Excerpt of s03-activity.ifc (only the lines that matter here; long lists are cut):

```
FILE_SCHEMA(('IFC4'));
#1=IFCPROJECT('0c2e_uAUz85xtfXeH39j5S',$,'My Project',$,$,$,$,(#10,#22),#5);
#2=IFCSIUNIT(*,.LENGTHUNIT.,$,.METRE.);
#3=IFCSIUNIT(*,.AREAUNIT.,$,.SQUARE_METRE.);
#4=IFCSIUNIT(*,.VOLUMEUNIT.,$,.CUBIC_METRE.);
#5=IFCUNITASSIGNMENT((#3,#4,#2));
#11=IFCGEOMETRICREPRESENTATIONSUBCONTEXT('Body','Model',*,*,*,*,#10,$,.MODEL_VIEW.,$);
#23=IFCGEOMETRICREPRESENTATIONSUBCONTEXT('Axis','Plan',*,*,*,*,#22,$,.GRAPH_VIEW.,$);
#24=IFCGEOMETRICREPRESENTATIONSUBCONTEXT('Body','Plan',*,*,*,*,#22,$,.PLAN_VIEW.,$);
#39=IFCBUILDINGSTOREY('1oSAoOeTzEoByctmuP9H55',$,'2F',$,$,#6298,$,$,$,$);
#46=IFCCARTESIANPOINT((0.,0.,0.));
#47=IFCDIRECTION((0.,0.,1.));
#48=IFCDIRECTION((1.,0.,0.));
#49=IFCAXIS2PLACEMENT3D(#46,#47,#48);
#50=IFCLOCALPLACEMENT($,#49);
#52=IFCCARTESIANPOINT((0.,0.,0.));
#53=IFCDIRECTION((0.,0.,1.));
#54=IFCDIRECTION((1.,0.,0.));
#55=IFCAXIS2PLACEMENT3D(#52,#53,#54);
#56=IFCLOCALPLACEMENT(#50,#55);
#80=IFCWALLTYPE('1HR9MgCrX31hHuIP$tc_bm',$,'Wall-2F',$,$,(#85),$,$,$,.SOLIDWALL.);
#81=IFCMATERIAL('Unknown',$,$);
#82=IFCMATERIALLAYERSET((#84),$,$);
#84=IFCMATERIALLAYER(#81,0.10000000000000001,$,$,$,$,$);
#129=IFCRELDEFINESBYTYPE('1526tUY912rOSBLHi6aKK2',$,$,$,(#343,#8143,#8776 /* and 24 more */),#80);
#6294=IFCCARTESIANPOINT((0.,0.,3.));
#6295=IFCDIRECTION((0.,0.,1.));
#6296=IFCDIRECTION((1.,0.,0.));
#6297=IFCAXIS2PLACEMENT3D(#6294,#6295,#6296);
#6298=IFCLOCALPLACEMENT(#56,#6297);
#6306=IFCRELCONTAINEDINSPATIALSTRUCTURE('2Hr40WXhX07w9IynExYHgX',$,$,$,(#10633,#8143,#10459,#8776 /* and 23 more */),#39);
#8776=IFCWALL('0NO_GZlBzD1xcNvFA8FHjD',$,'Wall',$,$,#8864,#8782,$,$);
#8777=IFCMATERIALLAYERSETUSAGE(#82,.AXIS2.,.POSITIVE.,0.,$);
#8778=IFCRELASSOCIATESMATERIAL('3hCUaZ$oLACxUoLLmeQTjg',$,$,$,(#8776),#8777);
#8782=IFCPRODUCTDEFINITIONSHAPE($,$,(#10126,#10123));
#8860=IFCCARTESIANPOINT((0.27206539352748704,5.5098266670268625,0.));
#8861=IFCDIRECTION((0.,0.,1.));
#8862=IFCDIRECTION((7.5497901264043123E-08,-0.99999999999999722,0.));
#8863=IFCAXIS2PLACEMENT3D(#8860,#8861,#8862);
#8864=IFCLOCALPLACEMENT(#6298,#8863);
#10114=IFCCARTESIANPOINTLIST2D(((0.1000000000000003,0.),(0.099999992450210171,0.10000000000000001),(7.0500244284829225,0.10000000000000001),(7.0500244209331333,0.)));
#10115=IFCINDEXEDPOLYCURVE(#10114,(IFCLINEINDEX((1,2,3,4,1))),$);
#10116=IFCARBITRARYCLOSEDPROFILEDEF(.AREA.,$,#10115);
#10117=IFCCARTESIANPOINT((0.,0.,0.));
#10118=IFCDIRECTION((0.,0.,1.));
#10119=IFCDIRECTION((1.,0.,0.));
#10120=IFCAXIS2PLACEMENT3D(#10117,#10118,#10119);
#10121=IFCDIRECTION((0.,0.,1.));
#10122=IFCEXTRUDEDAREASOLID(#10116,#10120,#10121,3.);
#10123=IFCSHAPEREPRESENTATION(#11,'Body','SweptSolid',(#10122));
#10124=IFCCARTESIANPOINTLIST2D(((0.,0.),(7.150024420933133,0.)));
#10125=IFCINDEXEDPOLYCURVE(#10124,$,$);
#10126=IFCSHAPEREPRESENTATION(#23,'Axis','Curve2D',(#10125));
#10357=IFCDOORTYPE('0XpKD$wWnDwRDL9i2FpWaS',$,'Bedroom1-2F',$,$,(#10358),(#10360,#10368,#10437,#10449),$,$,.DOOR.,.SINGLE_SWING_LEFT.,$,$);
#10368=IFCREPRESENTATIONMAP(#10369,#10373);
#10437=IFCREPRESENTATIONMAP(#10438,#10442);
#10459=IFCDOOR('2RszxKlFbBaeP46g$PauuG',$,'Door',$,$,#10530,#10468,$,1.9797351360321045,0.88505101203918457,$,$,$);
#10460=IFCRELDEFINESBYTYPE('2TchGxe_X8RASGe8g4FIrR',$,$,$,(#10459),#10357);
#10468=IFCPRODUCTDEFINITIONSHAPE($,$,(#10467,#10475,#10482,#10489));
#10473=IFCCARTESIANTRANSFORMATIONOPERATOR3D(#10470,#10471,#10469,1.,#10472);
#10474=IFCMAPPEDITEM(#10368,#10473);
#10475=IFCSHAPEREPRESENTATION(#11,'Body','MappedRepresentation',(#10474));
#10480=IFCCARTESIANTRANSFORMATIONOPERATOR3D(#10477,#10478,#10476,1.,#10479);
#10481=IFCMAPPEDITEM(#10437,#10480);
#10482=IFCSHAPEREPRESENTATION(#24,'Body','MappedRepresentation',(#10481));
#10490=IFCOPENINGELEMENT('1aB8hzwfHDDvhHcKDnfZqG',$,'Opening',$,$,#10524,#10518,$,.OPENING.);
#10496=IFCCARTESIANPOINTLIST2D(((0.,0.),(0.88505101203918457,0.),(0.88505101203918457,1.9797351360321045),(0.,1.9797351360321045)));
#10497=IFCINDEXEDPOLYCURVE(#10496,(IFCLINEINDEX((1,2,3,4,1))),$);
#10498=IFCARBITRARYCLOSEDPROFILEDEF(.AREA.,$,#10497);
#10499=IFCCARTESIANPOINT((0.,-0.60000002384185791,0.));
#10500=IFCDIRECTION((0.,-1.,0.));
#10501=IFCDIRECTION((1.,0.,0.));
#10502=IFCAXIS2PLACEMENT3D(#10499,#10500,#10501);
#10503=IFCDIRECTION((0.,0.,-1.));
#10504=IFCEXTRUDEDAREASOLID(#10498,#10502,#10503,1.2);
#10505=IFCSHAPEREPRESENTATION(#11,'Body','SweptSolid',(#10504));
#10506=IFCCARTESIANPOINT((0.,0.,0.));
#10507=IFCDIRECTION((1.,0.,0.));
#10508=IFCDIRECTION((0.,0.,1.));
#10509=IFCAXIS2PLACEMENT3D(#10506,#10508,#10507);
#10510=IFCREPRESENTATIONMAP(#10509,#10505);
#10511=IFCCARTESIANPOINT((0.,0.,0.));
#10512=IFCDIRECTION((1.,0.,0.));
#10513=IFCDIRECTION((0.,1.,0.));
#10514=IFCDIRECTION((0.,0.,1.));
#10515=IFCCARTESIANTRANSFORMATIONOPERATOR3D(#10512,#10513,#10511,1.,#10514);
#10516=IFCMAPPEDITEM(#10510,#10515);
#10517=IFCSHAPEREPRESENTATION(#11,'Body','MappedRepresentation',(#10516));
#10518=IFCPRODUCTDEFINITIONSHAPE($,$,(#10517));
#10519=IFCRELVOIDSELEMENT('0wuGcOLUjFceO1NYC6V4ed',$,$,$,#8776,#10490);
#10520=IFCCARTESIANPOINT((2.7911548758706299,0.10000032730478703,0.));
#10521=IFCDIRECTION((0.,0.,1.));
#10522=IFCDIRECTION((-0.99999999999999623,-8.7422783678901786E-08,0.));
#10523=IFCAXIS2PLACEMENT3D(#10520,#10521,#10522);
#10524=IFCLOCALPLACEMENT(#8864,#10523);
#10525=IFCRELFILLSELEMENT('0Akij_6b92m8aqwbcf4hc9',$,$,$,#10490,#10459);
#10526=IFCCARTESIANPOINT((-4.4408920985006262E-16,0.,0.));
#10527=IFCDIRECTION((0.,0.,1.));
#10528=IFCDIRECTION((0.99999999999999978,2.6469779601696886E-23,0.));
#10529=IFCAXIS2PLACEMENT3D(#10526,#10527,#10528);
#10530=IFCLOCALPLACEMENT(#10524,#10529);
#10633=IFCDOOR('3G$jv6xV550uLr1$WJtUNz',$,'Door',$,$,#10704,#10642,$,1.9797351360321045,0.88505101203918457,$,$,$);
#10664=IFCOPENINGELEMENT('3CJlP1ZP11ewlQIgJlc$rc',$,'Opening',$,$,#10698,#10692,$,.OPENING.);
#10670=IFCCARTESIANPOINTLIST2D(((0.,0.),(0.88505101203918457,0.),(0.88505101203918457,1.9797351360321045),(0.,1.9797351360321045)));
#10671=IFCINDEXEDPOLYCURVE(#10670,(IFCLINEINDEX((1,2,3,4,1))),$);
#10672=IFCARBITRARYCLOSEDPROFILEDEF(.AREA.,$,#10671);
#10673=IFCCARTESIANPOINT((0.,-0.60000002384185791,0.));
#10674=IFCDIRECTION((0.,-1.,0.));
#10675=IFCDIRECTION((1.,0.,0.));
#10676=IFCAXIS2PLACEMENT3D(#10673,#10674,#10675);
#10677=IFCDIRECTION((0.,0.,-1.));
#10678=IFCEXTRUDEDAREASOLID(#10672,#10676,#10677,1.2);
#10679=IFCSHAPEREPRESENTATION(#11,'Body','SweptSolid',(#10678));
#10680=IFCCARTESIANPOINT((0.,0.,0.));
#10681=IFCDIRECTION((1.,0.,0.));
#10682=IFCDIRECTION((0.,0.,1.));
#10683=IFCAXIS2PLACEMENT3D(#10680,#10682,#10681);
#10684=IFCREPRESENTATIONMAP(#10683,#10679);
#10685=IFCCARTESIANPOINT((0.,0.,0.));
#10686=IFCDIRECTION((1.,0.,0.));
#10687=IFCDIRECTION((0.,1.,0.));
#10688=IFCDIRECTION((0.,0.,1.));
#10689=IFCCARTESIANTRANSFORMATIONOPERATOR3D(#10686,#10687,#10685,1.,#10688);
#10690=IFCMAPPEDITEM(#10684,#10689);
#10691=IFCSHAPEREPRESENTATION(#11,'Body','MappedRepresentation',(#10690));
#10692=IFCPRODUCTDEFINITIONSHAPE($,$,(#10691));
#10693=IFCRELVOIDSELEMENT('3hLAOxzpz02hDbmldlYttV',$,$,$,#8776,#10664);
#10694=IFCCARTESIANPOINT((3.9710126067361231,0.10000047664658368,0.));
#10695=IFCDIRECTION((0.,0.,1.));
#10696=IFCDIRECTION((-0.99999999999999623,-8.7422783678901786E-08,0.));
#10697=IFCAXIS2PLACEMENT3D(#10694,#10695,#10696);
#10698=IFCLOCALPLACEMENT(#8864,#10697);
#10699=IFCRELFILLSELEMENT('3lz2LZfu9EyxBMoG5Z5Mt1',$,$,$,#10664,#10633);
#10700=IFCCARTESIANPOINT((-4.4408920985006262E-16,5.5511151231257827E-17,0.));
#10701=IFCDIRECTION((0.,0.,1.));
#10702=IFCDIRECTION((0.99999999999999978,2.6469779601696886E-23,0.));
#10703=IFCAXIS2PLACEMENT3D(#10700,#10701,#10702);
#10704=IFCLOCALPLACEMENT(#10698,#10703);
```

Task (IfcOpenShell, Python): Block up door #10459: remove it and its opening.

```python
import ifcopenshell
import ifcopenshell.api.feature
import ifcopenshell.api.root
import ifcopenshell.geom
import ifcopenshell.util.shape

model = ifcopenshell.open("s03-activity.ifc")
settings = ifcopenshell.geom.settings()


def volume(element):
    """Net volume in cubic metres, openings subtracted."""
    shape = ifcopenshell.geom.create_shape(settings, element)
    return ifcopenshell.util.shape.get_volume(shape.geometry)


door = model.by_guid("2RszxKlFbBaeP46g$PauuG")
opening = door.FillsVoids[0].RelatingOpeningElement
wall = opening.VoidsElements[0].RelatingBuildingElement
before = volume(wall)

ifcopenshell.api.root.remove_product(model, product=door)
ifcopenshell.api.feature.remove_feature(model, feature=opening)

after = volume(wall)

print(f"wall volume {before:.3f} -> {after:.3f} m3")

model.write("s03-activity_v2.ifc")
```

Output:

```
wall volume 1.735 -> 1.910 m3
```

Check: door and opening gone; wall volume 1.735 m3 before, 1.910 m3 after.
